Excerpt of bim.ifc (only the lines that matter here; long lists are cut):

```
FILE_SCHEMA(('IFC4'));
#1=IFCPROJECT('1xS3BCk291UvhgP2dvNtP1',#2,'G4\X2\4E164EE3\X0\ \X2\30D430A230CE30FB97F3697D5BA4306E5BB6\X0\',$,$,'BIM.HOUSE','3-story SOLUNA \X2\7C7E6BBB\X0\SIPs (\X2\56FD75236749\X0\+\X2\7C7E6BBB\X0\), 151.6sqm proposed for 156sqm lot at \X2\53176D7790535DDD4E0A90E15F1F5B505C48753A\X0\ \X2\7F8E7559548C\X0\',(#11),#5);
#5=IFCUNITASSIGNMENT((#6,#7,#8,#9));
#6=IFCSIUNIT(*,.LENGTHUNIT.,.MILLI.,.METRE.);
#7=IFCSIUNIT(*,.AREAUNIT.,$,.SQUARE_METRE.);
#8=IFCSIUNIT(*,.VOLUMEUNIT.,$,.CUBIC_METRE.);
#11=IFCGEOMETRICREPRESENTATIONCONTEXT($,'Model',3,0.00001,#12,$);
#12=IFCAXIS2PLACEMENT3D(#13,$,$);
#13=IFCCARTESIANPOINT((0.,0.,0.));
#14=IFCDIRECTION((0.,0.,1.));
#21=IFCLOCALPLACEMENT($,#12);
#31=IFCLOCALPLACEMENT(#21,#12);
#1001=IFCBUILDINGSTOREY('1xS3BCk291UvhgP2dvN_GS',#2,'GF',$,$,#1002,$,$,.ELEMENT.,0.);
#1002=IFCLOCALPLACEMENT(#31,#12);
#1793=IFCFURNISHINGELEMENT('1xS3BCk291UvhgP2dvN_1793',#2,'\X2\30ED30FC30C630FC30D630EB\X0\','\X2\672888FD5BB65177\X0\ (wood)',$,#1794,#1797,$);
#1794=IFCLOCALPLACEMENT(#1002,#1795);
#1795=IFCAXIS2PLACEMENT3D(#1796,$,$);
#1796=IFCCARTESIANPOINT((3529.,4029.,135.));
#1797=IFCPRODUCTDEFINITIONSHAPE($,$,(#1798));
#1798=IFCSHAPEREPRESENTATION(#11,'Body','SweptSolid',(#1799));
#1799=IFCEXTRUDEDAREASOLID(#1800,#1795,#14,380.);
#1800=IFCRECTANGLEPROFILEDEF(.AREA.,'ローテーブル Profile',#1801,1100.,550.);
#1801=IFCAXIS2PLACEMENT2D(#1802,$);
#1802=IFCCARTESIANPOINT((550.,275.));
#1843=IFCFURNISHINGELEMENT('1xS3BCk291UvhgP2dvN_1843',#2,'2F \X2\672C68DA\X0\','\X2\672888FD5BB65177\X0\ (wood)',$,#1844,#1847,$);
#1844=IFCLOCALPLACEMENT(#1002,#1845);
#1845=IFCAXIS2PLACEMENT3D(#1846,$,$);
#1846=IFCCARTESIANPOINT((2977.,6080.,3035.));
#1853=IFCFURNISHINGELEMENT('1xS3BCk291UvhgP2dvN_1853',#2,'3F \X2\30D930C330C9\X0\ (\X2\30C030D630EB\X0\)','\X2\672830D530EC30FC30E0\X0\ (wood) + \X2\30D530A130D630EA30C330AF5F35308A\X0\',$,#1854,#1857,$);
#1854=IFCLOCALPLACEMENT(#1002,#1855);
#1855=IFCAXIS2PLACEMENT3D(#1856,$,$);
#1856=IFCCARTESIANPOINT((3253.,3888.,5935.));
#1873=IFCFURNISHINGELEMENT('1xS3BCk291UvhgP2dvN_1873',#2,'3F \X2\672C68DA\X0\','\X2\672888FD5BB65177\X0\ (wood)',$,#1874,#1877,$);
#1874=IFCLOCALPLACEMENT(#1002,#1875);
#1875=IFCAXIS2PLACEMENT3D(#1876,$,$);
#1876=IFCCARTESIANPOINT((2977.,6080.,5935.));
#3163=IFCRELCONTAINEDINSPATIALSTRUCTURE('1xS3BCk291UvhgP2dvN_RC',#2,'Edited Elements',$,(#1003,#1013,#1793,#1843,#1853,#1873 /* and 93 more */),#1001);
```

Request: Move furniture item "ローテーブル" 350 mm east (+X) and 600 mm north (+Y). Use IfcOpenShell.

```python
import ifcopenshell
import ifcopenshell.api.geometry
import ifcopenshell.util.placement
import ifcopenshell.util.unit

model = ifcopenshell.open("bim.ifc")
unit_scale = ifcopenshell.util.unit.calculate_unit_scale(model)

item = model.by_guid("1xS3BCk291UvhgP2dvN_1793")
matrix = ifcopenshell.util.placement.get_local_placement(item.ObjectPlacement)
matrix[0, 3] += 0.35 / unit_scale
matrix[1, 3] += 0.6 / unit_scale
ifcopenshell.api.geometry.edit_object_placement(model, product=item, matrix=matrix, is_si=False)

print(ifcopenshell.util.placement.get_local_placement(item.ObjectPlacement).round(3) + 0.0)

model.write("bim_v2.ifc")
```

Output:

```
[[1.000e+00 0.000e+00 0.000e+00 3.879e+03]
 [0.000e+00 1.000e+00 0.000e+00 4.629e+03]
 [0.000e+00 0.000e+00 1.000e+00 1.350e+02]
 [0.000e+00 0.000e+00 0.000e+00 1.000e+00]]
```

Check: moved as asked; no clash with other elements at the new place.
